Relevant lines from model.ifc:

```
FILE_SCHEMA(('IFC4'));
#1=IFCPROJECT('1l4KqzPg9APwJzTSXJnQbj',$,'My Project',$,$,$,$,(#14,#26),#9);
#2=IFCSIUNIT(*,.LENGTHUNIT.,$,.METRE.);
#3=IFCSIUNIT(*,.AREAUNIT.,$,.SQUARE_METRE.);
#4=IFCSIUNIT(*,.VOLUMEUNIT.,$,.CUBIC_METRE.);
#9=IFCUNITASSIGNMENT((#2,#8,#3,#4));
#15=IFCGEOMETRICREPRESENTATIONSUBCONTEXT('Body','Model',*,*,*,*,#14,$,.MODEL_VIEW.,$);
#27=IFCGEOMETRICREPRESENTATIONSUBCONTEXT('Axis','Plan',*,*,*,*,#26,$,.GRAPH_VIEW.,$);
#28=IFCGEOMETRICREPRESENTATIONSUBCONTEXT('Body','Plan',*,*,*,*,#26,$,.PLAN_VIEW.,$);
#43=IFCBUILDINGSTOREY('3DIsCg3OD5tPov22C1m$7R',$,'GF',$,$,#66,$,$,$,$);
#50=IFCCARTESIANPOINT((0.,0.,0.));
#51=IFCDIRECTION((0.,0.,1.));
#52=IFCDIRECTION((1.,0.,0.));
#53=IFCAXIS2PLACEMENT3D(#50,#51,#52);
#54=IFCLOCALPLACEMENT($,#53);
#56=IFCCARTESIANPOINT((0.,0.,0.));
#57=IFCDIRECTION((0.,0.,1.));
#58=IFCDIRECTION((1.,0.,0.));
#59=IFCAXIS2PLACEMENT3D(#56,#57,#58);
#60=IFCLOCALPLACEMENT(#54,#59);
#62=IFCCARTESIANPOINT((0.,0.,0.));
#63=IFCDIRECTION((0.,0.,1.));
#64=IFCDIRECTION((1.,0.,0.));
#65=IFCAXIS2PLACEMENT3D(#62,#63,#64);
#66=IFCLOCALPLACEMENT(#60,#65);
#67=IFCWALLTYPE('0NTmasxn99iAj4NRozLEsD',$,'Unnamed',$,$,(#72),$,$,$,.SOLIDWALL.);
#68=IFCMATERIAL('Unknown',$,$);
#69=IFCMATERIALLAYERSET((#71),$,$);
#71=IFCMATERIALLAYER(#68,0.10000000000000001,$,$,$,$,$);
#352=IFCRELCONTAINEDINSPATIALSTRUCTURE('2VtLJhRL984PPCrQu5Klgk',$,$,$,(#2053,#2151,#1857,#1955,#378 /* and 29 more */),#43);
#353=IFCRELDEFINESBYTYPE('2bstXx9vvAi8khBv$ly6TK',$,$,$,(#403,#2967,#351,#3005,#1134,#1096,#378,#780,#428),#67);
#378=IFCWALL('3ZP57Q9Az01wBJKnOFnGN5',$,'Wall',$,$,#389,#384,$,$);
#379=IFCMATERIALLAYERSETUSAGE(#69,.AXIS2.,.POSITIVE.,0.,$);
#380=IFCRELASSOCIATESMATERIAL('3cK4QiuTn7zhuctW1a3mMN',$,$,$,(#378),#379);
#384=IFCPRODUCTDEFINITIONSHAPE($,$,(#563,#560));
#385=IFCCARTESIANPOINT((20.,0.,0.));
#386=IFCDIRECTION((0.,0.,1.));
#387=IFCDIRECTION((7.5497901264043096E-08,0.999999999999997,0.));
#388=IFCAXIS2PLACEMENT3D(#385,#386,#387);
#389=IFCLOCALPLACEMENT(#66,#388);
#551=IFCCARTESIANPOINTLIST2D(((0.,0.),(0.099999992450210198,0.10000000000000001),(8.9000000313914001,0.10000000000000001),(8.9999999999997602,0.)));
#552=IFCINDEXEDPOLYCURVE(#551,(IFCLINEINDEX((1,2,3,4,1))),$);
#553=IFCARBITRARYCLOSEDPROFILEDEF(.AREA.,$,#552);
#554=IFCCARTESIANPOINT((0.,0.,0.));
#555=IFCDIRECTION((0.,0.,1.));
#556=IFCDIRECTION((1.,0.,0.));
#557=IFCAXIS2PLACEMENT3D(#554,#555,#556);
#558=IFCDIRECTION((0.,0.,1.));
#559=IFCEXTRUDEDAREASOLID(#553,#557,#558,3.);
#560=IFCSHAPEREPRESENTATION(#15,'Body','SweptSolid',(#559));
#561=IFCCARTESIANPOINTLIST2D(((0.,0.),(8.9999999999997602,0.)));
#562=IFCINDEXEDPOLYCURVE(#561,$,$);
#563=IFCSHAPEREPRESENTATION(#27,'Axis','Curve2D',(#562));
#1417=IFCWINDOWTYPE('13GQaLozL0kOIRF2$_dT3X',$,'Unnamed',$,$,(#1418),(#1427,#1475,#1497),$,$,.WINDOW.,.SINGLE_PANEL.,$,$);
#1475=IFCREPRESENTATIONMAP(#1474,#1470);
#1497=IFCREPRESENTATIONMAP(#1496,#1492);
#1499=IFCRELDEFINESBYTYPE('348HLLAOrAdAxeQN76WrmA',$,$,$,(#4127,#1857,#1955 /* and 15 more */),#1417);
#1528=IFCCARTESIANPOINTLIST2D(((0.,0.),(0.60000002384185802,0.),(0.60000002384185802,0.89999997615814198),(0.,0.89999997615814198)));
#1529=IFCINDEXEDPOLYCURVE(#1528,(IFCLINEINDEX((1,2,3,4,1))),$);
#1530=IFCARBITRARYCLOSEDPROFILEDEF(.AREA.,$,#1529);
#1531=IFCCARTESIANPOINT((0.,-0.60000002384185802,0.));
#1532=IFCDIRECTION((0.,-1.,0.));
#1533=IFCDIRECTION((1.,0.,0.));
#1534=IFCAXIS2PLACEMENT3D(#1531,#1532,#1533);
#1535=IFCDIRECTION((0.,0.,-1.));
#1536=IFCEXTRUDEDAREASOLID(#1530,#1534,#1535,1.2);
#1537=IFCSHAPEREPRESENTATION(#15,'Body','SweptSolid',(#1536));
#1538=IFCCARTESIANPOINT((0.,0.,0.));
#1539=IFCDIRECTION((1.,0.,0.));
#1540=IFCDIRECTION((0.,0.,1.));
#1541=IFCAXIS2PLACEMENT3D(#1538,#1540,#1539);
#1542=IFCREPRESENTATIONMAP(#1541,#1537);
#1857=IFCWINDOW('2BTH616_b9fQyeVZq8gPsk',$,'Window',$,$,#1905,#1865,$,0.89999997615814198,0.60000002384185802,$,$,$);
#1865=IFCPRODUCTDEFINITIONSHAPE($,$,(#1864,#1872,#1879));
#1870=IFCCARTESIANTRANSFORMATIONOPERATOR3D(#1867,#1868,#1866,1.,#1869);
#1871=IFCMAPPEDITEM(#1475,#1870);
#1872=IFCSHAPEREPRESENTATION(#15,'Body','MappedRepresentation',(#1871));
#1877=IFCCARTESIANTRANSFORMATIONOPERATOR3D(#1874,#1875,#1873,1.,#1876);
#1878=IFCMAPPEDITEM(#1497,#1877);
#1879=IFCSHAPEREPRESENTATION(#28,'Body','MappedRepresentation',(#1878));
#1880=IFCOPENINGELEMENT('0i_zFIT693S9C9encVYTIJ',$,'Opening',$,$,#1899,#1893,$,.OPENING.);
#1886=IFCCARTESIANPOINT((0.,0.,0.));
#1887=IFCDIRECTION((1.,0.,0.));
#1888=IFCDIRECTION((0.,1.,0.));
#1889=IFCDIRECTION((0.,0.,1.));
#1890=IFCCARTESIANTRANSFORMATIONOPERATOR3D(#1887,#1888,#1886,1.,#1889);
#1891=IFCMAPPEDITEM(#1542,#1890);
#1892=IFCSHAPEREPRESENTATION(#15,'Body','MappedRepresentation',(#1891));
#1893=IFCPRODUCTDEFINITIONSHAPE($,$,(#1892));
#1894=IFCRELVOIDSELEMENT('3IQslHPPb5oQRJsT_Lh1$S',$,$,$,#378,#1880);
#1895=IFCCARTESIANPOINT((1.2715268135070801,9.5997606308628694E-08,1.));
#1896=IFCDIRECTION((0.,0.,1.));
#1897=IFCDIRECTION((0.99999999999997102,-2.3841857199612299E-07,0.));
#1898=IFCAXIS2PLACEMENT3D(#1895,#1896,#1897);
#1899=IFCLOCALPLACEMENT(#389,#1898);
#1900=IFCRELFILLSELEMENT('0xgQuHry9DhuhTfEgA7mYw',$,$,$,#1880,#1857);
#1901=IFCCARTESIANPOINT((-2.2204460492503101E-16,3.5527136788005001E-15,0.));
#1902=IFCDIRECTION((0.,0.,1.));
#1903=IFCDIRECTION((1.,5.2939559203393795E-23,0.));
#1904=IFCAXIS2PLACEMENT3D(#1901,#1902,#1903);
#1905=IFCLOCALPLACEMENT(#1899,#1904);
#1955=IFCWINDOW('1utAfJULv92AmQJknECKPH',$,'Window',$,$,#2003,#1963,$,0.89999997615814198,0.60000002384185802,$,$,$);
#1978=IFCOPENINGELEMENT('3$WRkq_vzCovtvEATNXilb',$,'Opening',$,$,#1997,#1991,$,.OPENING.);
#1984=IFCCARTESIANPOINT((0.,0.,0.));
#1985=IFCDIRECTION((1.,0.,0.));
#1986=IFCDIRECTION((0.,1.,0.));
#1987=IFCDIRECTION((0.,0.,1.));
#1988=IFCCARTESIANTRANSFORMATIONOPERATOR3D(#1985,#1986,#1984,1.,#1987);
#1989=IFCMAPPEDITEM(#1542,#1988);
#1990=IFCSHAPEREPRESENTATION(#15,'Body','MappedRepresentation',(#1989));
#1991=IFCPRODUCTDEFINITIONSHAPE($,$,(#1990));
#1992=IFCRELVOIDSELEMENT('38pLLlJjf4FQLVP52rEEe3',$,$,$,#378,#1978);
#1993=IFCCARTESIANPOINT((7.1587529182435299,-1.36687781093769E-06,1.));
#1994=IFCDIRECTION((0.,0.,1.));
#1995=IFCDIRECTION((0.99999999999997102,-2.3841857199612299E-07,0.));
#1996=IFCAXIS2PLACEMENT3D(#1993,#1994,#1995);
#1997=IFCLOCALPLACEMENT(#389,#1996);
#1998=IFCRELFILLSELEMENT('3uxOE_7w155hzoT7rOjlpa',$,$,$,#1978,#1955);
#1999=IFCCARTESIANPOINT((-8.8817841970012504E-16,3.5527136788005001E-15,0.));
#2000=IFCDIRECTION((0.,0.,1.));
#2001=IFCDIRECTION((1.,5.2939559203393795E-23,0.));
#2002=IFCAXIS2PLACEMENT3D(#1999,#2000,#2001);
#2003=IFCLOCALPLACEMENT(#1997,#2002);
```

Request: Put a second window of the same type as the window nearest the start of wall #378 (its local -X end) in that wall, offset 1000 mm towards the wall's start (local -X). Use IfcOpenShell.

```python
import ifcopenshell
import ifcopenshell.api.feature
import ifcopenshell.api.geometry
import ifcopenshell.api.root
import ifcopenshell.geom
import ifcopenshell.util.element
import ifcopenshell.util.placement
import ifcopenshell.util.shape
import ifcopenshell.util.unit

model = ifcopenshell.open("model.ifc")
unit_scale = ifcopenshell.util.unit.calculate_unit_scale(model)
settings = ifcopenshell.geom.settings()


def volume(element):
    """Net volume in cubic metres, openings subtracted."""
    shape = ifcopenshell.geom.create_shape(settings, element)
    return ifcopenshell.util.shape.get_volume(shape.geometry)


window = model.by_id(1857)
opening = window.FillsVoids[0].RelatingOpeningElement
wall = opening.VoidsElements[0].RelatingBuildingElement
before = volume(wall)
shift = ifcopenshell.util.placement.get_local_placement(wall.ObjectPlacement)[:3, 0] * -1 / unit_scale

# copy_class copies the void relationship, type, container and properties, but no geometry.
new_opening = ifcopenshell.api.root.copy_class(model, product=opening)
new_opening.Representation = ifcopenshell.util.element.copy_deep(
    model, opening.Representation, exclude=["IfcGeometricRepresentationContext", "IfcRepresentationMap"]
)
new_window = ifcopenshell.api.root.copy_class(model, product=window)
new_window.Representation = ifcopenshell.util.element.copy_deep(
    model, window.Representation, exclude=["IfcGeometricRepresentationContext", "IfcRepresentationMap"]
)
ifcopenshell.api.feature.add_filling(model, opening=new_opening, element=new_window)

for old, new in ((opening, new_opening), (window, new_window)):
    matrix = ifcopenshell.util.placement.get_local_placement(old.ObjectPlacement)
    matrix[:3, 3] += shift
    ifcopenshell.api.geometry.edit_object_placement(model, product=new, matrix=matrix, is_si=False)

after = volume(wall)

print(f"wall volume {before:.3f} -> {after:.3f} m3")

model.write("model_edited.ifc")
```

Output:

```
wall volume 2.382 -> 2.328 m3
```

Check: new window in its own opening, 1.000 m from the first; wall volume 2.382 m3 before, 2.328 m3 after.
